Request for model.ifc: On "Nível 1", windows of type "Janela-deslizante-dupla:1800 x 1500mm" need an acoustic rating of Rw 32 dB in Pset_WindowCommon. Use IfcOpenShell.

First a look at what the model holds.

```python
import ifcopenshell
import ifcopenshell.util.element

model = ifcopenshell.open("model.ifc")
print(model.schema)
storey = next(s for s in model.by_type("IfcBuildingStorey") if s.Name == "Nível 1")
windows = [e for e in ifcopenshell.util.element.get_decomposition(storey) if e.is_a("IfcWindow")]
seen = {}
for e in windows:
    element_type = ifcopenshell.util.element.get_type(e)
    key = (element_type.Name if element_type != e and element_type else None, ifcopenshell.util.element.get_pset(e, "Pset_WindowCommon", "AcousticRating"))
    seen[key] = seen.get(key, 0) + 1
for (name, value), count in sorted(seen.items(), key=str):
    print(count, "x", name, "|", value)
```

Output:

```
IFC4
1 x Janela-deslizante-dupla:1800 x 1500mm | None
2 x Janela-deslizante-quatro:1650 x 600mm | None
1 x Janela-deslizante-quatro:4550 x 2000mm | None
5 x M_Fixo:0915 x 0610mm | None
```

```python
import ifcopenshell
import ifcopenshell.api.pset
import ifcopenshell.util.element

model = ifcopenshell.open("model.ifc")

storey = next(s for s in model.by_type("IfcBuildingStorey") if s.Name == "Nível 1")
windows = [e for e in ifcopenshell.util.element.get_decomposition(storey) if e.is_a("IfcWindow")]

count = 0
for e in windows:
    element_type = ifcopenshell.util.element.get_type(e)
    if element_type in (None, e) or element_type.Name != "Janela-deslizante-dupla:1800 x 1500mm":
        continue
    # add_pset returns the element's existing set when there is one.
    pset = ifcopenshell.api.pset.add_pset(model, product=e, name="Pset_WindowCommon")
    ifcopenshell.api.pset.edit_pset(model, pset=pset, properties={"AcousticRating": "Rw 32 dB"})
    count += 1

print(count, "windows updated")

model.write("model-out.ifc")
```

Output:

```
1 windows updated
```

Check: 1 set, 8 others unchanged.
